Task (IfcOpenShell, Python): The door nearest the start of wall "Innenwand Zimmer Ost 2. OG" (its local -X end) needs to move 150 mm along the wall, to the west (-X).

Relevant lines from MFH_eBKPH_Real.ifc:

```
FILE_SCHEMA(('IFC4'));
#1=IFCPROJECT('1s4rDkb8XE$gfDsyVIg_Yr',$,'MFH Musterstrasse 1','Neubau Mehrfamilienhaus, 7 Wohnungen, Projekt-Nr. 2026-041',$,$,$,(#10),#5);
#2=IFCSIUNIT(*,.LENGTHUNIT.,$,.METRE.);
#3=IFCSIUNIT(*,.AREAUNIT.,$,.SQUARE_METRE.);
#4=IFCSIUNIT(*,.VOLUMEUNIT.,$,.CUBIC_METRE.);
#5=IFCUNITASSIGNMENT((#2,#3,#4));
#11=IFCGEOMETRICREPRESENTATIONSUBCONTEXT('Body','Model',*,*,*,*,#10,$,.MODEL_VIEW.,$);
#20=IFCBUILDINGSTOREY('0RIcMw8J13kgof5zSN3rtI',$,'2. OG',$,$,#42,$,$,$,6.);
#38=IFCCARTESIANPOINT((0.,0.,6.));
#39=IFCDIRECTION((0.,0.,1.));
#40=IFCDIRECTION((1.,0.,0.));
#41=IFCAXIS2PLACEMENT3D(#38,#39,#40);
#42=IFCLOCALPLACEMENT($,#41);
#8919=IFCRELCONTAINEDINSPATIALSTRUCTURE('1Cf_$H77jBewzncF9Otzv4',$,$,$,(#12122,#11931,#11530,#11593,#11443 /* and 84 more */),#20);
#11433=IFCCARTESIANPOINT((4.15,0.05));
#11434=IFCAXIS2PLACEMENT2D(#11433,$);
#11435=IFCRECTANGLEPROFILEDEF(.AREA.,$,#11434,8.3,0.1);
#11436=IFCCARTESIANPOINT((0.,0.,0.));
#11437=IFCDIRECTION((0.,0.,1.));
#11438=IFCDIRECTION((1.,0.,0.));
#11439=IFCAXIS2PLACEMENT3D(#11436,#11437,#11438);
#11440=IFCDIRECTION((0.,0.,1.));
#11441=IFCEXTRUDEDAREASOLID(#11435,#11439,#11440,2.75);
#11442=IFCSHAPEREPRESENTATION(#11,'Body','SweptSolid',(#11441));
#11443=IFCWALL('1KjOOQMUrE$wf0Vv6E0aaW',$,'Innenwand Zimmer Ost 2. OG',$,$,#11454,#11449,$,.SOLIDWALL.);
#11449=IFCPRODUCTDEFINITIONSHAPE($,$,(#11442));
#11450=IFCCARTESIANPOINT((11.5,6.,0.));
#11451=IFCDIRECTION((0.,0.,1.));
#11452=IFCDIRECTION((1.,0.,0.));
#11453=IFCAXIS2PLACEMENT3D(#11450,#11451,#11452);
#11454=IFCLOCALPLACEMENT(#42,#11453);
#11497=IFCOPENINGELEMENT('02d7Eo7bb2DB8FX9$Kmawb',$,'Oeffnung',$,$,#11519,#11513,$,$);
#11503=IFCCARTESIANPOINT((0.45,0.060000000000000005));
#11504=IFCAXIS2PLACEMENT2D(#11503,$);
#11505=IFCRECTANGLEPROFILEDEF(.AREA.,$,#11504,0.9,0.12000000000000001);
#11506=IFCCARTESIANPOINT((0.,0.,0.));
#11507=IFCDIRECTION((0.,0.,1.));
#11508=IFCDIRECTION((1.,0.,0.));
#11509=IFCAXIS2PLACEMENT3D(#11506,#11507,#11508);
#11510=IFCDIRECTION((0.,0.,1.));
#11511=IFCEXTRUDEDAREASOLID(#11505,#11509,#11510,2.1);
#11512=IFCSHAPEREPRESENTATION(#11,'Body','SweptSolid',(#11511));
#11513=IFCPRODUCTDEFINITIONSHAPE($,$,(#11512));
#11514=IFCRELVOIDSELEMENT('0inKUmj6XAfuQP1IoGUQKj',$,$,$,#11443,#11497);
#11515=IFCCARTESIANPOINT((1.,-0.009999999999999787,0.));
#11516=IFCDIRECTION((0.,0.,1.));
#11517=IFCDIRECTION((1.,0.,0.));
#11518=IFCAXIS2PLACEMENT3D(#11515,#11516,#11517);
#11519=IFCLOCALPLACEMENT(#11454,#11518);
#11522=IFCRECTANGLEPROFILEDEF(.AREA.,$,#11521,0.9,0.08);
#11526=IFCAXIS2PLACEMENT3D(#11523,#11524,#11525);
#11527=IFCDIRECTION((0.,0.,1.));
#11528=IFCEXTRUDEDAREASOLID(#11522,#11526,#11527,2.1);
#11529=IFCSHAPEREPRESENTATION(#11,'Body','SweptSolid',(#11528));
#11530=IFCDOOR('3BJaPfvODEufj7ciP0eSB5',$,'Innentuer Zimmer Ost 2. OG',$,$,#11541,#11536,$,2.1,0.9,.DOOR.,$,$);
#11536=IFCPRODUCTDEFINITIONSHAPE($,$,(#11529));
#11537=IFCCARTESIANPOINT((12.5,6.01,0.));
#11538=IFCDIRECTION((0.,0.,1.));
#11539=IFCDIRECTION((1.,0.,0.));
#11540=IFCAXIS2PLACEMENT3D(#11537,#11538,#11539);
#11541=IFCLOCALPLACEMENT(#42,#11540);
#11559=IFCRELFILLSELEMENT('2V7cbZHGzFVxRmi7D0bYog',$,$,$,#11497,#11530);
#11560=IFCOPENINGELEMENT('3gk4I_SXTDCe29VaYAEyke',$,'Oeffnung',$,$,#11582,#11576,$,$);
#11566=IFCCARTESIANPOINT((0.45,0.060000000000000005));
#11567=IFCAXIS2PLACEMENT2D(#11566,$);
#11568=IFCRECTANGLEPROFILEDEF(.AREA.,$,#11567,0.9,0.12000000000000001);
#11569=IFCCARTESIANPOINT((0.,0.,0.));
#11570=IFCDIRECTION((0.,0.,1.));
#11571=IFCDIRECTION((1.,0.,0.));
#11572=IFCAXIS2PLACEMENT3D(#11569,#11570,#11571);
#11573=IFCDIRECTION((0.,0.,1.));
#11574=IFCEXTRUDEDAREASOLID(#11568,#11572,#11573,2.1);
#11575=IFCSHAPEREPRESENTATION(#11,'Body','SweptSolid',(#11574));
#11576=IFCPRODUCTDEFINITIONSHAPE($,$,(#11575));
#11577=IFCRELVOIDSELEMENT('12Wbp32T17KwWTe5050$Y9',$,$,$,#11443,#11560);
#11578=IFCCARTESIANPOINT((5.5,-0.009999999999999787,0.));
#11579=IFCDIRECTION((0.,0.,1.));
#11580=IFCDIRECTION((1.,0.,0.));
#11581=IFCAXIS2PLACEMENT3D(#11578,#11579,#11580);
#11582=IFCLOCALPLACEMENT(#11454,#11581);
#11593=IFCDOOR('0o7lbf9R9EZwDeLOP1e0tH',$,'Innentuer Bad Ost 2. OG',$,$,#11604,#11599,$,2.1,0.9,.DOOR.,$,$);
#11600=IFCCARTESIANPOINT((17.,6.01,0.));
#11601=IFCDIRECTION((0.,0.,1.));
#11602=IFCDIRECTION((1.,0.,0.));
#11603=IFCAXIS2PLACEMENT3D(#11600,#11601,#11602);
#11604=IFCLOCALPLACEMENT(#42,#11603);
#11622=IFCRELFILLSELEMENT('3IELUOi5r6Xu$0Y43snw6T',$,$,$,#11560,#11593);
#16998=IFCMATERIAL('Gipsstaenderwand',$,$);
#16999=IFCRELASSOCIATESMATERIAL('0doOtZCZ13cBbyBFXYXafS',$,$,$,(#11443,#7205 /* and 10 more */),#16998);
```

```python
import ifcopenshell
import ifcopenshell.api.geometry
import ifcopenshell.util.placement

model = ifcopenshell.open("MFH_eBKPH_Real.ifc")

door = model.by_guid("3BJaPfvODEufj7ciP0eSB5")
opening = door.FillsVoids[0].RelatingOpeningElement
wall = opening.VoidsElements[0].RelatingBuildingElement

wall_matrix = ifcopenshell.util.placement.get_local_placement(wall.ObjectPlacement)
shift = wall_matrix[:3, 0] * -0.15
before = ifcopenshell.util.placement.get_local_placement(door.ObjectPlacement)[:3, 3].copy()

# The door is not placed relative to its opening, so move both.
for product in (opening, door):
    matrix = ifcopenshell.util.placement.get_local_placement(product.ObjectPlacement)
    matrix[:3, 3] += shift
    ifcopenshell.api.geometry.edit_object_placement(model, product=product, matrix=matrix, is_si=False)

after = ifcopenshell.util.placement.get_local_placement(door.ObjectPlacement)[:3, 3]
print("door moved by", (after - before).round(3) + 0.0)

model.write("MFH_eBKPH_Real_edited.ifc")
```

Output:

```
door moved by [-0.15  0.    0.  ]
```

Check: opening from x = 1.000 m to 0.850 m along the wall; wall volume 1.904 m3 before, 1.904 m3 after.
